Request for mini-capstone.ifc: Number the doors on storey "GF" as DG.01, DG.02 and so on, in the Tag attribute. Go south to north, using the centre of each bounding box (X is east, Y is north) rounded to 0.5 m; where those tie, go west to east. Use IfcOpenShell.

First a look at what the model holds.

```python
import ifcopenshell
import ifcopenshell.util.element
import ifcopenshell.util.placement

model = ifcopenshell.open("mini-capstone.ifc")
print(model.schema)
storey = next(s for s in model.by_type("IfcBuildingStorey") if s.Name == "GF")
doors = [e for e in ifcopenshell.util.element.get_decomposition(storey) if e.is_a("IfcDoor")]
for e in sorted(doors, key=lambda e: e.id()):
    origin = ifcopenshell.util.placement.get_local_placement(e.ObjectPlacement)[:3, 3]
    print(e.id(), e.Tag, e.Name, origin.round(2) + 0.0, sep=" | ")
```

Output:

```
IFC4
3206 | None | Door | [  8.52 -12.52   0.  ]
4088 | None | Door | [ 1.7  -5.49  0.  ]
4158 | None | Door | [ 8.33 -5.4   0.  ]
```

```python
import ifcopenshell
import ifcopenshell.geom
import ifcopenshell.util.element
import ifcopenshell.util.shape

model = ifcopenshell.open("mini-capstone.ifc")
settings = ifcopenshell.geom.settings()
settings.set("use-world-coords", True)


def centre(element):
    shape = ifcopenshell.geom.create_shape(settings, element)
    return ifcopenshell.util.shape.get_bbox_centroid(shape.geometry)


storey = next(s for s in model.by_type("IfcBuildingStorey") if s.Name == "GF")
doors = [e for e in ifcopenshell.util.element.get_decomposition(storey) if e.is_a("IfcDoor")]

# Insertion points can sit at a corner or the storey origin, so sort by the geometry (in metres).
centres = {e: centre(e) for e in doors}
doors.sort(key=lambda e: (round(centres[e][1] / 0.5), centres[e][0]))

for i, e in enumerate(doors, start=1):
    number = f"DG.{i:02d}"
    e.Tag = number
    print(e.id(), number)

model.write("mini-capstone_updated.ifc")
```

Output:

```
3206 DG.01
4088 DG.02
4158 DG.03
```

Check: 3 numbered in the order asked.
